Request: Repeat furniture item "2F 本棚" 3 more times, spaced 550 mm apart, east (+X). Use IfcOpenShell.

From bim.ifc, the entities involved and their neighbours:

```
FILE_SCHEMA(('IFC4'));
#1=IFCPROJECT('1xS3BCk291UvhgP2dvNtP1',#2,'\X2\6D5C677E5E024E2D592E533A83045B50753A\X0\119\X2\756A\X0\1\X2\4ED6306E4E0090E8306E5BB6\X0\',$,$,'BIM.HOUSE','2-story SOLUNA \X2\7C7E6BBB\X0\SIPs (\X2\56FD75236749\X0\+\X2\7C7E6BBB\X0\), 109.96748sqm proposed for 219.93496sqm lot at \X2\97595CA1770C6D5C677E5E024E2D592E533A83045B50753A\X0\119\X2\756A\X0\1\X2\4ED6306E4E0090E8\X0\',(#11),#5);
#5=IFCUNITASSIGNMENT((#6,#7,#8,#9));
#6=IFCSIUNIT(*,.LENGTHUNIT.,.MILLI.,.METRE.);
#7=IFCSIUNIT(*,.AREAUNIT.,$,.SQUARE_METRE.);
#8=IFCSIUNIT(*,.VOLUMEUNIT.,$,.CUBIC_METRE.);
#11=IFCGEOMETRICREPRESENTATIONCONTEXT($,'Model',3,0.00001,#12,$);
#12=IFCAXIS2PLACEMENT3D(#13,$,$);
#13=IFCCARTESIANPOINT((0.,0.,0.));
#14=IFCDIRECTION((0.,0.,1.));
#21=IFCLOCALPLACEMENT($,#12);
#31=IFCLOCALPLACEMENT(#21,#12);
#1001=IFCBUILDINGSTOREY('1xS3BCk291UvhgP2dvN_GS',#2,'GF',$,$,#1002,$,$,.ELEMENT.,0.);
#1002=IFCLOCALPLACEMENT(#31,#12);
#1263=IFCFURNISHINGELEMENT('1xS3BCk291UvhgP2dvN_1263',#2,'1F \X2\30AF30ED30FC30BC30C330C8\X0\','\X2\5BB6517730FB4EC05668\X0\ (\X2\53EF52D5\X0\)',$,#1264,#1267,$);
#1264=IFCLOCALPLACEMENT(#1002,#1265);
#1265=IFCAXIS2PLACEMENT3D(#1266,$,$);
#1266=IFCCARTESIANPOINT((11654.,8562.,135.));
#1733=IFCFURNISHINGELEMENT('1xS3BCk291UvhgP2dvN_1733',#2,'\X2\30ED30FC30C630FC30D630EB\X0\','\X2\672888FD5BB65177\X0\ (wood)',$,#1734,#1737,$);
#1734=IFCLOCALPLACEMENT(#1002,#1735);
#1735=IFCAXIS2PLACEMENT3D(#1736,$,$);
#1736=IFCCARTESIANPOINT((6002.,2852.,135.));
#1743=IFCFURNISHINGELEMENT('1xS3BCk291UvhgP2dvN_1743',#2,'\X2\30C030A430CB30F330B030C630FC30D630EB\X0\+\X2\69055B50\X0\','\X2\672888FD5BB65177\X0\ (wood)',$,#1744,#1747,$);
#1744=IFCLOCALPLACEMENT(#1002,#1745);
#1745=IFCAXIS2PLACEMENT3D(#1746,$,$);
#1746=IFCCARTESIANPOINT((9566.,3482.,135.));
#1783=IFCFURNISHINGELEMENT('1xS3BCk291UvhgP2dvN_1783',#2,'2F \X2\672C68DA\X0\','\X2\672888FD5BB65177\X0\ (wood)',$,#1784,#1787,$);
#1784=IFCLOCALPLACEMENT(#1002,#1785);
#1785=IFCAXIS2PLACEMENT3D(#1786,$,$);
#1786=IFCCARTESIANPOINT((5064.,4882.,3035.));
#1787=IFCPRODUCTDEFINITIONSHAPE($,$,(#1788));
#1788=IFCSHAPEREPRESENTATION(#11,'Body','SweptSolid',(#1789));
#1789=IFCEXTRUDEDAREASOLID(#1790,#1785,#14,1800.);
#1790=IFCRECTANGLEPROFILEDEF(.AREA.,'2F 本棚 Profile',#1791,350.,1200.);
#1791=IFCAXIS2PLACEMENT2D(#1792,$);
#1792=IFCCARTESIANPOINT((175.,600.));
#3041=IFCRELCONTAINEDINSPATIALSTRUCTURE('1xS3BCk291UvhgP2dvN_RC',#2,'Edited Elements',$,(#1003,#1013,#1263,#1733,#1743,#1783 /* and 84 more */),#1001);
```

```python
import numpy as np
import ifcopenshell
import ifcopenshell.api.geometry
import ifcopenshell.api.root
import ifcopenshell.util.element
import ifcopenshell.util.placement

model = ifcopenshell.open("bim.ifc")


def reuse_history(source, copy):
    """copy_class also copies each property set's owner history, people and application; keep the originals."""
    for rel in copy.IsDefinedBy:
        if rel.is_a("IfcRelDefinesByProperties") and (history := rel.RelatingPropertyDefinition.OwnerHistory):
            rel.RelatingPropertyDefinition.OwnerHistory = source.OwnerHistory
            ifcopenshell.util.element.remove_deep2(model, history)


source = model.by_guid("1xS3BCk291UvhgP2dvN_1783")
base = ifcopenshell.util.placement.get_local_placement(source.ObjectPlacement)
step = np.array([1.0, 0.0, 0.0]) * 550.0

for i in range(1, 4):
    copy = ifcopenshell.api.root.copy_class(model, product=source)
    copy.Representation = ifcopenshell.util.element.copy_deep(
        model, source.Representation, exclude=["IfcGeometricRepresentationContext", "IfcRepresentationMap"]
    )
    reuse_history(source, copy)
    matrix = base.copy()
    matrix[:3, 3] += i * step
    print("added at", matrix[:3, 3].round(3) + 0.0)
    ifcopenshell.api.geometry.edit_object_placement(model, product=copy, matrix=matrix, is_si=False)

model.write("bim_v2.ifc")
```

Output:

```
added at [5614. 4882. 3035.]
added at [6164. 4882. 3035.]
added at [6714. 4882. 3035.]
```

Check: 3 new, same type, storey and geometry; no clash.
